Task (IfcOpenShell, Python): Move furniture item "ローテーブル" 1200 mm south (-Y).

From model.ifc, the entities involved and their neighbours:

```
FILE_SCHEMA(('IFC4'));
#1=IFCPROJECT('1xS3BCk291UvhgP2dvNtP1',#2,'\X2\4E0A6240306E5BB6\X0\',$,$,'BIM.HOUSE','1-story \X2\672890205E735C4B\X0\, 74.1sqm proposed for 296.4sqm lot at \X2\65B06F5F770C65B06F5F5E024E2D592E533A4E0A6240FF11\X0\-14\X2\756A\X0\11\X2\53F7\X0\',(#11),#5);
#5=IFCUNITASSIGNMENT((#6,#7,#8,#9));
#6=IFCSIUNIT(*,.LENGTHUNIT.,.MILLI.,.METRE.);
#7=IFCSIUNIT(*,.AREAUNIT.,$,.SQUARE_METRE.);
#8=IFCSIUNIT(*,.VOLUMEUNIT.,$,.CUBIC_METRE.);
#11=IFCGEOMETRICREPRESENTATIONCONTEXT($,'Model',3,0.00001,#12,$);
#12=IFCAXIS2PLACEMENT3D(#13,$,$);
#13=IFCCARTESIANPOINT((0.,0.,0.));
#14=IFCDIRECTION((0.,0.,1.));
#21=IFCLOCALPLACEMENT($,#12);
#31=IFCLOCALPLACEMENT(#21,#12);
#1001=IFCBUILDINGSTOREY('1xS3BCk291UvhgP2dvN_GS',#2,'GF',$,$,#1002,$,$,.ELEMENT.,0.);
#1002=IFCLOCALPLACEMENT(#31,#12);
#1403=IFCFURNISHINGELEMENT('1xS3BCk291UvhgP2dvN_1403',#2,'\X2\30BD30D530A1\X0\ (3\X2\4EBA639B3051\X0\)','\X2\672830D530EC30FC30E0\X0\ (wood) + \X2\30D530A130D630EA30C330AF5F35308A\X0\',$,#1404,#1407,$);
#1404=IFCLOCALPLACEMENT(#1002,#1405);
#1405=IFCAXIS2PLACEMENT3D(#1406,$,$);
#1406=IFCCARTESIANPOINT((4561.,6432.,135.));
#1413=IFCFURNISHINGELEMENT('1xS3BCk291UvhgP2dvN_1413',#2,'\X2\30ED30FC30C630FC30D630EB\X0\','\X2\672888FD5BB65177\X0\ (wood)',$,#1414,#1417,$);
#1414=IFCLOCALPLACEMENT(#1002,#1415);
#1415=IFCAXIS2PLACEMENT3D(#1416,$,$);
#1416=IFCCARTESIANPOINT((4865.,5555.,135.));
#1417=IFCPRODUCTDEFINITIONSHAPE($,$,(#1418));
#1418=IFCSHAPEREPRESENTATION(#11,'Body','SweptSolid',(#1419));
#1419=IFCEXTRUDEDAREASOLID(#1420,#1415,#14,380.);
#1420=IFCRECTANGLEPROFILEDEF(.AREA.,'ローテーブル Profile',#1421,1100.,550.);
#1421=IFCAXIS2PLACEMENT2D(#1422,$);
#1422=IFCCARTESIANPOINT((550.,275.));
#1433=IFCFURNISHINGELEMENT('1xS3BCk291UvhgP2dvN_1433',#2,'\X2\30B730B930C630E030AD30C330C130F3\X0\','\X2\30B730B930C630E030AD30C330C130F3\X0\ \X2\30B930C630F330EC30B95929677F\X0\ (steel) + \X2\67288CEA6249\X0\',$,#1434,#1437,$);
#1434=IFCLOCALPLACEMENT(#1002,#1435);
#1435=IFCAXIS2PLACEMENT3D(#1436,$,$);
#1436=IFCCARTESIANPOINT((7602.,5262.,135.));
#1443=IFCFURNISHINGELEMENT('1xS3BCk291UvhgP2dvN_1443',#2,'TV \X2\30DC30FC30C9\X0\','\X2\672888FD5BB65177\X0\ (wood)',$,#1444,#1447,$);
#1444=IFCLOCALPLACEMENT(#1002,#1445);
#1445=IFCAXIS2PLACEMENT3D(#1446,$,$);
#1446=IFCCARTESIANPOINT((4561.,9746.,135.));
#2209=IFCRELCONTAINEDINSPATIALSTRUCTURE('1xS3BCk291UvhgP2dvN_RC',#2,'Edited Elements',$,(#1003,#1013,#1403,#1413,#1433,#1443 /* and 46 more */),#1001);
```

```python
import ifcopenshell
import ifcopenshell.api.geometry
import ifcopenshell.util.placement

model = ifcopenshell.open("model.ifc")

item = model.by_id(1413)
matrix = ifcopenshell.util.placement.get_local_placement(item.ObjectPlacement)
matrix[1, 3] -= 1200.0
ifcopenshell.api.geometry.edit_object_placement(model, product=item, matrix=matrix, is_si=False)

print(ifcopenshell.util.placement.get_local_placement(item.ObjectPlacement).round(3) + 0.0)

model.write("model_v2.ifc")
```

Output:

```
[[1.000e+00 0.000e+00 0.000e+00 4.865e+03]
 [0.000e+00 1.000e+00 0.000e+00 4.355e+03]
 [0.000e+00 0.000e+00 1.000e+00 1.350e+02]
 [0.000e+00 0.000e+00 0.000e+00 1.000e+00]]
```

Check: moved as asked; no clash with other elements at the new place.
